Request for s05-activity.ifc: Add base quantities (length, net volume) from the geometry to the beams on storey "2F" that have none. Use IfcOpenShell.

First a look at what the model holds.

```python
import ifcopenshell
import ifcopenshell.util.element
import ifcopenshell.util.unit

model = ifcopenshell.open("s05-activity.ifc")
print(model.schema)
for unit_type in ("LENGTHUNIT", "AREAUNIT", "VOLUMEUNIT"):
    print(unit_type, ifcopenshell.util.unit.calculate_unit_scale(model, unit_type))
storey = next(s for s in model.by_type("IfcBuildingStorey") if s.Name == "2F")
beams = [e for e in ifcopenshell.util.element.get_decomposition(storey) if e.is_a("IfcBeam")]
for e in sorted(beams, key=lambda e: e.id()):
    print(e.id(), e.is_a(), e.Name, list(ifcopenshell.util.element.get_psets(e, qtos_only=True)), sep=" | ")
```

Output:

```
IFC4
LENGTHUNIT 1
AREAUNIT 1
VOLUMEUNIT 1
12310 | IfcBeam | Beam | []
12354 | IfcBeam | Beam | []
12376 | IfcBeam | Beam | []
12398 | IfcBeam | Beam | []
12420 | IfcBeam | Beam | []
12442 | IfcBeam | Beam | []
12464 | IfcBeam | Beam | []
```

```python
import ifcopenshell
import ifcopenshell.api.pset
import ifcopenshell.geom
import ifcopenshell.util.element
import ifcopenshell.util.shape
import ifcopenshell.util.unit

model = ifcopenshell.open("s05-activity.ifc")
unit_scale = ifcopenshell.util.unit.calculate_unit_scale(model)
volume_scale = ifcopenshell.util.unit.calculate_unit_scale(model, "VOLUMEUNIT")
settings = ifcopenshell.geom.settings()

storey = next(s for s in model.by_type("IfcBuildingStorey") if s.Name == "2F")
beams = [e for e in ifcopenshell.util.element.get_decomposition(storey) if e.is_a("IfcBeam")]

for e in sorted(beams, key=lambda e: e.id()):
    if ifcopenshell.util.element.get_psets(e, qtos_only=True, should_inherit=False):
        continue
    # Geometry comes back in metres, in the element's own axes.
    shape = ifcopenshell.geom.create_shape(settings, e)
    values = {
        "Length": ifcopenshell.util.shape.get_max_xyz(shape.geometry) / unit_scale,
        "NetVolume": ifcopenshell.util.shape.get_volume(shape.geometry) / volume_scale,
    }
    qto = ifcopenshell.api.pset.add_qto(model, product=e, name="Qto_BeamBaseQuantities")
    ifcopenshell.api.pset.edit_qto(model, qto=qto, properties=values)
    print(e.id(), {k: round(v, 3) for k, v in values.items()})

model.write("s05-activity-out.ifc")
```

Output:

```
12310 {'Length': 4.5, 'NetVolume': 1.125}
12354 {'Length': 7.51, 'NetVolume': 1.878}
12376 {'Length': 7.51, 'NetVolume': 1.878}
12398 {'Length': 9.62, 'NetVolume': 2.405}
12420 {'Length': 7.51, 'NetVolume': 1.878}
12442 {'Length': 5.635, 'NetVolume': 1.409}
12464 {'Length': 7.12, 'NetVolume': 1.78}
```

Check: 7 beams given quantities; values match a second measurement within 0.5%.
